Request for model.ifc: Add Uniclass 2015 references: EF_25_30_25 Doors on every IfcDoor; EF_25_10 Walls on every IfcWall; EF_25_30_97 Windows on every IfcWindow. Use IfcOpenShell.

First a look at what the model holds.

```python
import ifcopenshell

model = ifcopenshell.open("model.ifc")
print(model.schema)
print("classifications:", [c.Name for c in model.by_type("IfcClassification")])
for ifc_class in ("IfcDoor", "IfcRoof", "IfcStair", "IfcWall", "IfcWindow"):
    print(ifc_class, len(model.by_type(ifc_class)))
```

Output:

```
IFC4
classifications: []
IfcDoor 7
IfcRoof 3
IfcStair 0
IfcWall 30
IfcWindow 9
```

```python
import ifcopenshell
import ifcopenshell.api.classification

model = ifcopenshell.open("model.ifc")

system = ifcopenshell.api.classification.add_classification(model, classification="Uniclass 2015")

codes = {
    "IfcDoor": ("EF_25_30_25", "Doors"),
    "IfcWall": ("EF_25_10", "Walls"),
    "IfcWindow": ("EF_25_30_97", "Windows"),
}
for ifc_class, (code, name) in codes.items():
    products = model.by_type(ifc_class)
    ifcopenshell.api.classification.add_reference(
        model, products=products, classification=system, identification=code, name=name
    )
    print(code, len(products))

model.write("model_v2.ifc")
```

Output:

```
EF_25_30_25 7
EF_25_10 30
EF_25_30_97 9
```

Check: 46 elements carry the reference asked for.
